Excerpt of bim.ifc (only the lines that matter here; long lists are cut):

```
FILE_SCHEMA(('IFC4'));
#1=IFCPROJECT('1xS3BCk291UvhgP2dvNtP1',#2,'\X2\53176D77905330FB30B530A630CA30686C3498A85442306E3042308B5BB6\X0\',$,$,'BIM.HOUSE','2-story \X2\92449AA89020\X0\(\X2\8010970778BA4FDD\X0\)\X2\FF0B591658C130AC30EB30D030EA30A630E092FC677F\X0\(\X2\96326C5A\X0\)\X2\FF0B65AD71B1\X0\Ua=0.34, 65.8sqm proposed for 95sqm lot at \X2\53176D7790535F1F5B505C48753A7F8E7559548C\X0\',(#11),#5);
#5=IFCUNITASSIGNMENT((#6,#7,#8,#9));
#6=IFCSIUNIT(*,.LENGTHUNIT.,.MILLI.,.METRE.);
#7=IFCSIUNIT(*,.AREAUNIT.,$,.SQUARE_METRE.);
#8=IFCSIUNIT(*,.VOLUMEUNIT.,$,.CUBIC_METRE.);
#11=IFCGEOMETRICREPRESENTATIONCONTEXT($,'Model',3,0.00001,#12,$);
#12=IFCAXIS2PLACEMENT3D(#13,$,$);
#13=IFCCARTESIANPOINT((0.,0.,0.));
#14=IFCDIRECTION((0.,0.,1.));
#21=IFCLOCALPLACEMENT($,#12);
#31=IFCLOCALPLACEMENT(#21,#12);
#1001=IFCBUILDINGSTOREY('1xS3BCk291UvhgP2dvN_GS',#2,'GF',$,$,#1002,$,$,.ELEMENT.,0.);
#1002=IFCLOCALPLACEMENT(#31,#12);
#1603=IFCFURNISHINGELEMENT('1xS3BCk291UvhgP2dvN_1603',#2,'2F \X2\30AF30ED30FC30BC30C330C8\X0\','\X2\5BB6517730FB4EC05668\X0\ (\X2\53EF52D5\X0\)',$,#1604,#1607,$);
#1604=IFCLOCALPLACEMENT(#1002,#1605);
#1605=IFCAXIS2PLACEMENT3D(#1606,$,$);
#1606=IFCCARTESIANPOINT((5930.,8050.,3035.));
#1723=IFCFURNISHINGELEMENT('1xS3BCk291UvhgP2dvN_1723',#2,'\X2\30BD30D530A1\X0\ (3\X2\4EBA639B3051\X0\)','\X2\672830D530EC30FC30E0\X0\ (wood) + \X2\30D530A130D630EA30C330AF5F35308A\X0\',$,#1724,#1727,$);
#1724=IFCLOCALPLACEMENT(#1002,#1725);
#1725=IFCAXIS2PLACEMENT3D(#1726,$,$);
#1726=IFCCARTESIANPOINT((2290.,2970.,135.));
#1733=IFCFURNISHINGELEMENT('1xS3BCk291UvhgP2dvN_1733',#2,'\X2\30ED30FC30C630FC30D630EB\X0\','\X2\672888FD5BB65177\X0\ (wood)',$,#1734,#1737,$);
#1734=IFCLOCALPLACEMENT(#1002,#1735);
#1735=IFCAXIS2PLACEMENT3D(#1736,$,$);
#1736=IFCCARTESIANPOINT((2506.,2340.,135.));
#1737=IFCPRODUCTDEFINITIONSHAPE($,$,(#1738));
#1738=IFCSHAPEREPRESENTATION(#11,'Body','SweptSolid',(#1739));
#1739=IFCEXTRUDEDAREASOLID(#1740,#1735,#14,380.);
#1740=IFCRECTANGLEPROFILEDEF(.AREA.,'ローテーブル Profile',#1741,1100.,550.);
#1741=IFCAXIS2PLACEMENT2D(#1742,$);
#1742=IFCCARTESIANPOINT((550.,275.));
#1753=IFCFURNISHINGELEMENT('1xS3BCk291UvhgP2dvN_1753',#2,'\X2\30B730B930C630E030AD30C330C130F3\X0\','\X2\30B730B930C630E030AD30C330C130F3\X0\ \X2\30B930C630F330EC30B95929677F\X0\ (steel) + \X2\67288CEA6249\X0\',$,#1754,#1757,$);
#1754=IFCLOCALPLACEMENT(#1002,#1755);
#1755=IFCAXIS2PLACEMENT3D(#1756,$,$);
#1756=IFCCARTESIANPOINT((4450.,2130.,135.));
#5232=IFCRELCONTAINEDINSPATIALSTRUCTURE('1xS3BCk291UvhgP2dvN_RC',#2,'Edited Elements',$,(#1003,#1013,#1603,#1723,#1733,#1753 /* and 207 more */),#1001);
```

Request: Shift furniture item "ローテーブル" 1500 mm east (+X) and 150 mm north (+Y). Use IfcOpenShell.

```python
import ifcopenshell
import ifcopenshell.api.geometry
import ifcopenshell.util.placement

model = ifcopenshell.open("bim.ifc")

item = model.by_guid("1xS3BCk291UvhgP2dvN_1733")
matrix = ifcopenshell.util.placement.get_local_placement(item.ObjectPlacement)
matrix[0, 3] += 1500.0
matrix[1, 3] += 150.0
ifcopenshell.api.geometry.edit_object_placement(model, product=item, matrix=matrix, is_si=False)

print(ifcopenshell.util.placement.get_local_placement(item.ObjectPlacement).round(3) + 0.0)

model.write("bim_updated.ifc")
```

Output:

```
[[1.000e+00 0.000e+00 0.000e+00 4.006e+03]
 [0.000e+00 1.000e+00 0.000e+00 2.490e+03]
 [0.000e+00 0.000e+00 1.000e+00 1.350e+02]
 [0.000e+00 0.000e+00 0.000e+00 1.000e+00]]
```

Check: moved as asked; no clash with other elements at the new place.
